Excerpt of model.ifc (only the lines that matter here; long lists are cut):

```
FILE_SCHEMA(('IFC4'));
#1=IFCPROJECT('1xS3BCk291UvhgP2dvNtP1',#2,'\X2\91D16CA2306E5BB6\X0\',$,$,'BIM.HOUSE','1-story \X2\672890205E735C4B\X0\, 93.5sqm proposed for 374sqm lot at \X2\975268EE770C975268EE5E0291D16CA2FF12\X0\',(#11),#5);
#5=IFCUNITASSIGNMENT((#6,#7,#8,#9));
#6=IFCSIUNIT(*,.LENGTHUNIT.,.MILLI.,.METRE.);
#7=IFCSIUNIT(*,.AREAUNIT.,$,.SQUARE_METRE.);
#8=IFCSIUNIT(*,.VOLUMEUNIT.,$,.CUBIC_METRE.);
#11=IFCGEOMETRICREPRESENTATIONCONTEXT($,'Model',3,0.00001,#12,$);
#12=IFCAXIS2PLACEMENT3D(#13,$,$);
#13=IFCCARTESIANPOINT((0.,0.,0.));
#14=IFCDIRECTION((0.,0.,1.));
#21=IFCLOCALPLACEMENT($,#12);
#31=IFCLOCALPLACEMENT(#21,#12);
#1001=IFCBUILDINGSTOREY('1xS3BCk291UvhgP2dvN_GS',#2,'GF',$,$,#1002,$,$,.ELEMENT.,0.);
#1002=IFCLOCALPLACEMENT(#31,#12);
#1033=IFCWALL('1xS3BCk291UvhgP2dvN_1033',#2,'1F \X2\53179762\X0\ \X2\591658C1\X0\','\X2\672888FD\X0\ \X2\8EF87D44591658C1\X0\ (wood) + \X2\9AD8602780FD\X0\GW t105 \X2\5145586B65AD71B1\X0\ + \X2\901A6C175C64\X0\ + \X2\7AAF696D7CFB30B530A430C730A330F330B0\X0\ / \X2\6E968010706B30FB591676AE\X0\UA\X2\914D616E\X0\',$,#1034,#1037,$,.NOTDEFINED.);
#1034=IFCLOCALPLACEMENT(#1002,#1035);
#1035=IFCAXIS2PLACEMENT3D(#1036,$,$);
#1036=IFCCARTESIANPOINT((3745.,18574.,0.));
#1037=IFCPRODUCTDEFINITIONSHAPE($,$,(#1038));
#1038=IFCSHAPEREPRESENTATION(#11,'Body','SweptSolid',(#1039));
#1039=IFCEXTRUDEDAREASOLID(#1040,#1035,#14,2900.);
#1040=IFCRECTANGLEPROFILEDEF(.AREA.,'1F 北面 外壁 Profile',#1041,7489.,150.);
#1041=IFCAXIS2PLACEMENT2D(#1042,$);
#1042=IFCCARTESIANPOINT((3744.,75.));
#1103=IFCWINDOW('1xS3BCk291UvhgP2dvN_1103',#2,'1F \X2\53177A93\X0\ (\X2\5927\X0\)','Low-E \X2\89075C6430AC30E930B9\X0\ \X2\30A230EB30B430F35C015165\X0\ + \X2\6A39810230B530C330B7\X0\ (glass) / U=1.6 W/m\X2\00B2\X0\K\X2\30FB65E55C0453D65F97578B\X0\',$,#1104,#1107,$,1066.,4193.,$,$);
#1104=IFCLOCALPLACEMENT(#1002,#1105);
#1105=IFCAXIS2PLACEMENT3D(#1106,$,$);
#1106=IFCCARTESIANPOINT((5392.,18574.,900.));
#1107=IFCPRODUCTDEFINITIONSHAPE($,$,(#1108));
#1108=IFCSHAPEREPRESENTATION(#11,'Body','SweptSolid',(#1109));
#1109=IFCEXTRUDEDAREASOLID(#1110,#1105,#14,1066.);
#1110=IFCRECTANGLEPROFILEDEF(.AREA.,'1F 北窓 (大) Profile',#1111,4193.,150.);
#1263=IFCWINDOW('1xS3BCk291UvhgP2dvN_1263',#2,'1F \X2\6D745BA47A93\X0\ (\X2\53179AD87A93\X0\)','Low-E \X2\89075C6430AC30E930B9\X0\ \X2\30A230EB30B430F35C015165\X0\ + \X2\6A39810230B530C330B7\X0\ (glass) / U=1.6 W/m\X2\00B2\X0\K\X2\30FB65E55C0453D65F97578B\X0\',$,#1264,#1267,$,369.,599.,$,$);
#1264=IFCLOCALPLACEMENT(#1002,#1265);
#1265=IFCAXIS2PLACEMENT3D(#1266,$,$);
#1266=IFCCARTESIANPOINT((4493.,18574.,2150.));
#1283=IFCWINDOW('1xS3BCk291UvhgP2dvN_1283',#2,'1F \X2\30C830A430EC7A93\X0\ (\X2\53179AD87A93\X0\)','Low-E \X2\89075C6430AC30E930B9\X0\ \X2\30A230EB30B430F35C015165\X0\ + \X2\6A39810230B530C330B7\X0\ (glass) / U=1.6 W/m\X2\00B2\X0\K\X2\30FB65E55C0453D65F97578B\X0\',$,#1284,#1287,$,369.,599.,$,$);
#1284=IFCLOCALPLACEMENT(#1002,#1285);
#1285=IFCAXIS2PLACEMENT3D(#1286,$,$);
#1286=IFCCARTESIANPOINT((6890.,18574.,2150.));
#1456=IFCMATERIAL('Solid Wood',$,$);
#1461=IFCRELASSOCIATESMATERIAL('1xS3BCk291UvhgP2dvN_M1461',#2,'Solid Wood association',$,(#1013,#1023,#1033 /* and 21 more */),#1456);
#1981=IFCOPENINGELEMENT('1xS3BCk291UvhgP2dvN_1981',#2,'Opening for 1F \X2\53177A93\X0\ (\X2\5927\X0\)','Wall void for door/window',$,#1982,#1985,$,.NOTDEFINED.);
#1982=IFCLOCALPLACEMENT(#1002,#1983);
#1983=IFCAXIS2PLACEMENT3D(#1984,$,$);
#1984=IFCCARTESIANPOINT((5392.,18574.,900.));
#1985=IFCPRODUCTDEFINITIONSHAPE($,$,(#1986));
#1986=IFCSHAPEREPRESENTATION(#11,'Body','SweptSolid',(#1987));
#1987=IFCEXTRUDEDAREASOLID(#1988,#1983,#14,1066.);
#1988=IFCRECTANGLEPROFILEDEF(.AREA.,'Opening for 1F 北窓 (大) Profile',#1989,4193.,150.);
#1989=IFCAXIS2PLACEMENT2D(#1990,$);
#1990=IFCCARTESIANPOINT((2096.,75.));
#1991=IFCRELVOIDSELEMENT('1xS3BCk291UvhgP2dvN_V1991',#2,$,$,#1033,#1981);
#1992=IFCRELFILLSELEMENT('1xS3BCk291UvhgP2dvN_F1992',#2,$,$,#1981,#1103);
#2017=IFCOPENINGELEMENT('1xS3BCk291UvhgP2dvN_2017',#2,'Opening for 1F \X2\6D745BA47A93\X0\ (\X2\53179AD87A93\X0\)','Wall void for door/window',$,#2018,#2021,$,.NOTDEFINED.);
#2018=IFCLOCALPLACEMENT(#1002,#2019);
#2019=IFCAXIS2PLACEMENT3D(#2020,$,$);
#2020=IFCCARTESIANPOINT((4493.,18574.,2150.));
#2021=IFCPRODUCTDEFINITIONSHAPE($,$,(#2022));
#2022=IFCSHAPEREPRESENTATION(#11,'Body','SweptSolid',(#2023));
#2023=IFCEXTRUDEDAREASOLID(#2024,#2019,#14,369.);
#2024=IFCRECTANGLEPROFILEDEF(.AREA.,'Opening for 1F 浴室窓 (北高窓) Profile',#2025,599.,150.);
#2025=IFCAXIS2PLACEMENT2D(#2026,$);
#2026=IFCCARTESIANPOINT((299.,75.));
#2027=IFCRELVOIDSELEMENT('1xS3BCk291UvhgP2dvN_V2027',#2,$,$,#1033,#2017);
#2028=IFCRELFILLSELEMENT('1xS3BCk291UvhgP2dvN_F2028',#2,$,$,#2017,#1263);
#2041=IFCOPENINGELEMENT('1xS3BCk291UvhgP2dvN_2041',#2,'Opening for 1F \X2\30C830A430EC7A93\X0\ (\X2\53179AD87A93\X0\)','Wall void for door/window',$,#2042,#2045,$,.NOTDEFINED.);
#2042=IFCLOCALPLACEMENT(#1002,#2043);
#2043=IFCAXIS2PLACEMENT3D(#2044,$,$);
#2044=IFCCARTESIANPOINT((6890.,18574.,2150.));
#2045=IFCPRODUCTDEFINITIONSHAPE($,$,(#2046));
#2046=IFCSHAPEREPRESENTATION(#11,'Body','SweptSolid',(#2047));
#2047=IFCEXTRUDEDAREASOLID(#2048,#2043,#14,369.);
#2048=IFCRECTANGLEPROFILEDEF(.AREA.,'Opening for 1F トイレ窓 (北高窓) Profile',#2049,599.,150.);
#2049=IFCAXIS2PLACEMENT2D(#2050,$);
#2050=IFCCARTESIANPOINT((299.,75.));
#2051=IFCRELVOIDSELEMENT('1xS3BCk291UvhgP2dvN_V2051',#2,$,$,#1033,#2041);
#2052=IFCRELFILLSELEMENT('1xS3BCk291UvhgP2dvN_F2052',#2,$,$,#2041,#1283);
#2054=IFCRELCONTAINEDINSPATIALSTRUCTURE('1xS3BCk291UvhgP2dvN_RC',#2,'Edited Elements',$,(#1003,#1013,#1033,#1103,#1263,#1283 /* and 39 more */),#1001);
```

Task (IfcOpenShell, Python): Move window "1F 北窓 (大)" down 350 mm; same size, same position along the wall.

```python
import numpy as np
import ifcopenshell
import ifcopenshell.api.geometry
import ifcopenshell.util.placement
import ifcopenshell.util.unit

model = ifcopenshell.open("model.ifc")
unit_scale = ifcopenshell.util.unit.calculate_unit_scale(model)

window = model.by_id(1103)
opening = window.FillsVoids[0].RelatingOpeningElement
dz = -350.0

shift = np.array([0.0, 0.0, dz])
# The window is not placed relative to its opening, so move both.
for product in (opening, window):
    matrix = ifcopenshell.util.placement.get_local_placement(product.ObjectPlacement)
    matrix[:3, 3] += shift
    ifcopenshell.api.geometry.edit_object_placement(model, product=product, matrix=matrix, is_si=False)

print(f"moved by {dz * unit_scale:+.3f} m")

model.write("model_v2.ifc")
```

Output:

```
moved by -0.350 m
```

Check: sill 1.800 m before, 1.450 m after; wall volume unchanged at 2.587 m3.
